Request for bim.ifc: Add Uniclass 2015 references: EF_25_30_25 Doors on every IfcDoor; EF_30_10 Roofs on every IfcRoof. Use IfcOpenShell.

First a look at what the model holds.

```python
import ifcopenshell

model = ifcopenshell.open("bim.ifc")
print(model.schema)
print("classifications:", [c.Name for c in model.by_type("IfcClassification")])
for ifc_class in ("IfcDoor", "IfcRoof", "IfcStair", "IfcWall", "IfcWindow"):
    print(ifc_class, len(model.by_type(ifc_class)))
```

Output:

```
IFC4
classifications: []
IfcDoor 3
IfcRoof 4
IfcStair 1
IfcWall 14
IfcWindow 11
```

```python
import ifcopenshell
import ifcopenshell.api.classification

model = ifcopenshell.open("bim.ifc")

system = ifcopenshell.api.classification.add_classification(model, classification="Uniclass 2015")

codes = {
    "IfcDoor": ("EF_25_30_25", "Doors"),
    "IfcRoof": ("EF_30_10", "Roofs"),
}
for ifc_class, (code, name) in codes.items():
    products = model.by_type(ifc_class)
    ifcopenshell.api.classification.add_reference(
        model, products=products, classification=system, identification=code, name=name
    )
    print(code, len(products))

model.write("bim_edited.ifc")
```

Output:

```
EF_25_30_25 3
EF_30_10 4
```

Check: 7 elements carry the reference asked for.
